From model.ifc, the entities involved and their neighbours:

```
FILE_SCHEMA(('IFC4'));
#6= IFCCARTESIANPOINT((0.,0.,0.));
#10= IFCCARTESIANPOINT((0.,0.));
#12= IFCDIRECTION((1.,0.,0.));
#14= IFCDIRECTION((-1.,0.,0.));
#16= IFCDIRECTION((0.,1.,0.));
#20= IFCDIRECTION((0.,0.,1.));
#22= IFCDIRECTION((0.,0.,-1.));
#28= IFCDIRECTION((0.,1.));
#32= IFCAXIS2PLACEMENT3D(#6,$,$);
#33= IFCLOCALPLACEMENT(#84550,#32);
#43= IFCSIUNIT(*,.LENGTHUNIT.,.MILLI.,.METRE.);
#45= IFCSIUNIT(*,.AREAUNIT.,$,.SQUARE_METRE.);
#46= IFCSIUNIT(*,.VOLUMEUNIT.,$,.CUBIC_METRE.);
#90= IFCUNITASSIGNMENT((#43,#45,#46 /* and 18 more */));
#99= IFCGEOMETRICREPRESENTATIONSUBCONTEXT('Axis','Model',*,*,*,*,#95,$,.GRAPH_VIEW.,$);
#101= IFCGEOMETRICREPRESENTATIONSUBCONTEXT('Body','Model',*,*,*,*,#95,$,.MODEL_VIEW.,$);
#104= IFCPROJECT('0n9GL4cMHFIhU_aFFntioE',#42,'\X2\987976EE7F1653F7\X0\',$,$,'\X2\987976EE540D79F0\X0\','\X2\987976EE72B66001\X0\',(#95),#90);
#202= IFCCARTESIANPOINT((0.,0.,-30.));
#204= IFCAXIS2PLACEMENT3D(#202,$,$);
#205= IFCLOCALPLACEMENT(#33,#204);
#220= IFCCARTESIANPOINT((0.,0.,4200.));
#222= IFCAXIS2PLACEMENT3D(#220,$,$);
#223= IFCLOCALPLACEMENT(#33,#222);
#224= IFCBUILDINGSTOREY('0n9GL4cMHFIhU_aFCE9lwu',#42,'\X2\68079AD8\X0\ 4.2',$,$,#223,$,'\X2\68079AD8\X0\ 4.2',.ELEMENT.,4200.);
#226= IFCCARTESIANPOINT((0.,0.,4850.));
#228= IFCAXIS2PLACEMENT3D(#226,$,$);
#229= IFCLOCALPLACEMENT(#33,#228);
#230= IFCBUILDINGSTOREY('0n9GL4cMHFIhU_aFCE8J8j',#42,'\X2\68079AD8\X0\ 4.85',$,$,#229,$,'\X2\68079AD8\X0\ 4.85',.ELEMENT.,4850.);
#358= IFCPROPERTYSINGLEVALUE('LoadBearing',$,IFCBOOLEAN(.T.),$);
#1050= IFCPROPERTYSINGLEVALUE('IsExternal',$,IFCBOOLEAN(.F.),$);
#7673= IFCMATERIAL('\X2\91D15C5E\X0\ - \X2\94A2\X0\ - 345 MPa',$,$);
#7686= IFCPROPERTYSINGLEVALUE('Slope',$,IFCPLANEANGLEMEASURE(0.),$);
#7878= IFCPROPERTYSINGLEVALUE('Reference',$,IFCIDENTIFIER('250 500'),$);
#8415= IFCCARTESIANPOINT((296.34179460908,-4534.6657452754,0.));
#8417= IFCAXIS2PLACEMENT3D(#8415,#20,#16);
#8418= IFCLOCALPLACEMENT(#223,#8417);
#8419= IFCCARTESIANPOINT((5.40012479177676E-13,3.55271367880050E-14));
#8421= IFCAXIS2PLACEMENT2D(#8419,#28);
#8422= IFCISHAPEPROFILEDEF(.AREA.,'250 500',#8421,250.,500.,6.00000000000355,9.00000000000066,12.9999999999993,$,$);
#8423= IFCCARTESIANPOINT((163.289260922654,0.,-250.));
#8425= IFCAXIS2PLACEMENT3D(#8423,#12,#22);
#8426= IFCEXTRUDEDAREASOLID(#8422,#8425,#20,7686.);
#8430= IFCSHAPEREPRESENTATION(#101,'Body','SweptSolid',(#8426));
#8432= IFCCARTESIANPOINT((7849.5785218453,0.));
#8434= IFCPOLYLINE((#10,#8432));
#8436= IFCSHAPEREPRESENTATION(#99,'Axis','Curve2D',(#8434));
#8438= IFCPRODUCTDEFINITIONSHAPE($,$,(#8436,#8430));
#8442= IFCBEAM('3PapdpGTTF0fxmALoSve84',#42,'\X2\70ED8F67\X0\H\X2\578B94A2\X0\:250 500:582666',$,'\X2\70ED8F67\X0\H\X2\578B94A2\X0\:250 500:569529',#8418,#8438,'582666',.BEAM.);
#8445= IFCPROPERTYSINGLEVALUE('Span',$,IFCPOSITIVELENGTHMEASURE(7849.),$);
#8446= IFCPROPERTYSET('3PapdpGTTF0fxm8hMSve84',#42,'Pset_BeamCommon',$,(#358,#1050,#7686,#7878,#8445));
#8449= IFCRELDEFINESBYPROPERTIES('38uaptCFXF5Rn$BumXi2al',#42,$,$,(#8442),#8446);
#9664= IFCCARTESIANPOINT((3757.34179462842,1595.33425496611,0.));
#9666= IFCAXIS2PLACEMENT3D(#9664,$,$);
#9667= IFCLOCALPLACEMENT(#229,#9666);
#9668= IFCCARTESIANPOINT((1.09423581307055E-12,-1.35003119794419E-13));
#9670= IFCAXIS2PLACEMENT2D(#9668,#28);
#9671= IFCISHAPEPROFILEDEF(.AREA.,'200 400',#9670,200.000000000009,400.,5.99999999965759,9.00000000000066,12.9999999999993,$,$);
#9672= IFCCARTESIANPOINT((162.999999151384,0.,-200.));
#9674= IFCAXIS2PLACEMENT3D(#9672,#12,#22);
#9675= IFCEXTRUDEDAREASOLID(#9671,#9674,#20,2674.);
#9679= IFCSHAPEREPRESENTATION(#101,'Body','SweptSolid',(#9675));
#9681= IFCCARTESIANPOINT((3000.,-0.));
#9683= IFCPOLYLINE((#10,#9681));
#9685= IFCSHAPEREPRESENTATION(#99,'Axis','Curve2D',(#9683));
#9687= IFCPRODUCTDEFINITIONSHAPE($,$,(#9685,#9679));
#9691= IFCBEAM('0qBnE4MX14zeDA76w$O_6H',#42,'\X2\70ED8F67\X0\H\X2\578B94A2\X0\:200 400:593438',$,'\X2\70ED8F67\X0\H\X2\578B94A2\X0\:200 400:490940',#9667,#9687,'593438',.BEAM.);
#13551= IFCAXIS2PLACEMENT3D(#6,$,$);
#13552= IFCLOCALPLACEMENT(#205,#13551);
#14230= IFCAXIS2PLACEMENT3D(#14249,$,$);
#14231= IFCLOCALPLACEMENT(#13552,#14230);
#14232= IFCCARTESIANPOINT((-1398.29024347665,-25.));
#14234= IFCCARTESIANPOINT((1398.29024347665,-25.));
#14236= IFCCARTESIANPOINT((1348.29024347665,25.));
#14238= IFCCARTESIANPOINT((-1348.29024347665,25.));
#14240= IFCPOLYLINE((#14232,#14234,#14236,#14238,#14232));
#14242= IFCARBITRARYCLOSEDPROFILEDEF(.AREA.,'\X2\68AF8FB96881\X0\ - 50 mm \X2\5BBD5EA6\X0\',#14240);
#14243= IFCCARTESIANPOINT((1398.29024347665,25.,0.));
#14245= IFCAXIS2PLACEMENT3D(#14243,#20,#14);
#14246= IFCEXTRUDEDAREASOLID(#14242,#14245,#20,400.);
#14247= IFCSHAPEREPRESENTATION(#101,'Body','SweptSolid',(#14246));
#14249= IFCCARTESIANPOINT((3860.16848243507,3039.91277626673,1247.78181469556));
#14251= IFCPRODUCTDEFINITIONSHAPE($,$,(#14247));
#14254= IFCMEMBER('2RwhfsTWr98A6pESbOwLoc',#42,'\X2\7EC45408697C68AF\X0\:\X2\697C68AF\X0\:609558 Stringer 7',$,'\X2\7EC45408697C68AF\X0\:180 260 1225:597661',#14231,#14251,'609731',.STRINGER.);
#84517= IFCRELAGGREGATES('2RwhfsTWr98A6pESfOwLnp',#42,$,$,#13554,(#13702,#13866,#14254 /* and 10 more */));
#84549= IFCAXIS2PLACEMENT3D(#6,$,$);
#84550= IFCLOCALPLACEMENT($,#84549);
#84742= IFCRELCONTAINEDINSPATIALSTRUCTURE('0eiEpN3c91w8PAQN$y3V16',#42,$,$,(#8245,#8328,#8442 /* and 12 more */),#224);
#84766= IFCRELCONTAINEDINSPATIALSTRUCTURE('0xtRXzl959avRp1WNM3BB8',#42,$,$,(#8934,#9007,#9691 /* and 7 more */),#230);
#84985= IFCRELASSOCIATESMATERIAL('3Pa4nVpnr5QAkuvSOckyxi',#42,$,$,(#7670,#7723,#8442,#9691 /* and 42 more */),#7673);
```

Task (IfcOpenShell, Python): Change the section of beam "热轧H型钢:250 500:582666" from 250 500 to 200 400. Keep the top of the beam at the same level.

```python
import ifcopenshell
import ifcopenshell.api.pset
import ifcopenshell.util.element
import ifcopenshell.util.representation

model = ifcopenshell.open("model.ifc")

member = model.by_guid("3PapdpGTTF0fxmALoSve84")
source = next(p for p in model.by_type("IfcIShapeProfileDef") if p.ProfileName == "200 400")

body = ifcopenshell.util.representation.get_representation(member, "Model", "Body")
solid = body.Items[0]
old_profile = solid.SweptArea

# Copy the section's sizes but keep this member's own profile position.
profile = ifcopenshell.util.element.copy(model, source)
# Profiles are centred, so shift by half the change in depth to hold the top.
shift = (old_profile.OverallDepth - profile.OverallDepth) / 2
x, y = old_profile.Position.Location.Coordinates
up = (-1.0, 0.0)  # upwards, in the solid's own plane
location = model.createIfcCartesianPoint((x + up[0] * shift, y + up[1] * shift))
profile.Position = model.createIfcAxis2Placement2D(location, old_profile.Position.RefDirection)
solid.SweptArea = profile
if not model.get_total_inverses(old_profile):
    ifcopenshell.util.element.remove_deep2(model, old_profile)
member.Name = member.Name.replace("250 500", "200 400")
member.ObjectType = member.ObjectType.replace("250 500", "200 400")
pset = model.by_id(ifcopenshell.util.element.get_pset(member, "Pset_BeamCommon", should_inherit=False)["id"])
ifcopenshell.api.pset.edit_pset(model, pset=pset, properties={"Reference": "200 400"})

print(solid.SweptArea)

model.write("model_edited.ifc")
```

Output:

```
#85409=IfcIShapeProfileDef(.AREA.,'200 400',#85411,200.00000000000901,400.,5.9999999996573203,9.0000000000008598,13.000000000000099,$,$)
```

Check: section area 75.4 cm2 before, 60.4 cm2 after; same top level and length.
